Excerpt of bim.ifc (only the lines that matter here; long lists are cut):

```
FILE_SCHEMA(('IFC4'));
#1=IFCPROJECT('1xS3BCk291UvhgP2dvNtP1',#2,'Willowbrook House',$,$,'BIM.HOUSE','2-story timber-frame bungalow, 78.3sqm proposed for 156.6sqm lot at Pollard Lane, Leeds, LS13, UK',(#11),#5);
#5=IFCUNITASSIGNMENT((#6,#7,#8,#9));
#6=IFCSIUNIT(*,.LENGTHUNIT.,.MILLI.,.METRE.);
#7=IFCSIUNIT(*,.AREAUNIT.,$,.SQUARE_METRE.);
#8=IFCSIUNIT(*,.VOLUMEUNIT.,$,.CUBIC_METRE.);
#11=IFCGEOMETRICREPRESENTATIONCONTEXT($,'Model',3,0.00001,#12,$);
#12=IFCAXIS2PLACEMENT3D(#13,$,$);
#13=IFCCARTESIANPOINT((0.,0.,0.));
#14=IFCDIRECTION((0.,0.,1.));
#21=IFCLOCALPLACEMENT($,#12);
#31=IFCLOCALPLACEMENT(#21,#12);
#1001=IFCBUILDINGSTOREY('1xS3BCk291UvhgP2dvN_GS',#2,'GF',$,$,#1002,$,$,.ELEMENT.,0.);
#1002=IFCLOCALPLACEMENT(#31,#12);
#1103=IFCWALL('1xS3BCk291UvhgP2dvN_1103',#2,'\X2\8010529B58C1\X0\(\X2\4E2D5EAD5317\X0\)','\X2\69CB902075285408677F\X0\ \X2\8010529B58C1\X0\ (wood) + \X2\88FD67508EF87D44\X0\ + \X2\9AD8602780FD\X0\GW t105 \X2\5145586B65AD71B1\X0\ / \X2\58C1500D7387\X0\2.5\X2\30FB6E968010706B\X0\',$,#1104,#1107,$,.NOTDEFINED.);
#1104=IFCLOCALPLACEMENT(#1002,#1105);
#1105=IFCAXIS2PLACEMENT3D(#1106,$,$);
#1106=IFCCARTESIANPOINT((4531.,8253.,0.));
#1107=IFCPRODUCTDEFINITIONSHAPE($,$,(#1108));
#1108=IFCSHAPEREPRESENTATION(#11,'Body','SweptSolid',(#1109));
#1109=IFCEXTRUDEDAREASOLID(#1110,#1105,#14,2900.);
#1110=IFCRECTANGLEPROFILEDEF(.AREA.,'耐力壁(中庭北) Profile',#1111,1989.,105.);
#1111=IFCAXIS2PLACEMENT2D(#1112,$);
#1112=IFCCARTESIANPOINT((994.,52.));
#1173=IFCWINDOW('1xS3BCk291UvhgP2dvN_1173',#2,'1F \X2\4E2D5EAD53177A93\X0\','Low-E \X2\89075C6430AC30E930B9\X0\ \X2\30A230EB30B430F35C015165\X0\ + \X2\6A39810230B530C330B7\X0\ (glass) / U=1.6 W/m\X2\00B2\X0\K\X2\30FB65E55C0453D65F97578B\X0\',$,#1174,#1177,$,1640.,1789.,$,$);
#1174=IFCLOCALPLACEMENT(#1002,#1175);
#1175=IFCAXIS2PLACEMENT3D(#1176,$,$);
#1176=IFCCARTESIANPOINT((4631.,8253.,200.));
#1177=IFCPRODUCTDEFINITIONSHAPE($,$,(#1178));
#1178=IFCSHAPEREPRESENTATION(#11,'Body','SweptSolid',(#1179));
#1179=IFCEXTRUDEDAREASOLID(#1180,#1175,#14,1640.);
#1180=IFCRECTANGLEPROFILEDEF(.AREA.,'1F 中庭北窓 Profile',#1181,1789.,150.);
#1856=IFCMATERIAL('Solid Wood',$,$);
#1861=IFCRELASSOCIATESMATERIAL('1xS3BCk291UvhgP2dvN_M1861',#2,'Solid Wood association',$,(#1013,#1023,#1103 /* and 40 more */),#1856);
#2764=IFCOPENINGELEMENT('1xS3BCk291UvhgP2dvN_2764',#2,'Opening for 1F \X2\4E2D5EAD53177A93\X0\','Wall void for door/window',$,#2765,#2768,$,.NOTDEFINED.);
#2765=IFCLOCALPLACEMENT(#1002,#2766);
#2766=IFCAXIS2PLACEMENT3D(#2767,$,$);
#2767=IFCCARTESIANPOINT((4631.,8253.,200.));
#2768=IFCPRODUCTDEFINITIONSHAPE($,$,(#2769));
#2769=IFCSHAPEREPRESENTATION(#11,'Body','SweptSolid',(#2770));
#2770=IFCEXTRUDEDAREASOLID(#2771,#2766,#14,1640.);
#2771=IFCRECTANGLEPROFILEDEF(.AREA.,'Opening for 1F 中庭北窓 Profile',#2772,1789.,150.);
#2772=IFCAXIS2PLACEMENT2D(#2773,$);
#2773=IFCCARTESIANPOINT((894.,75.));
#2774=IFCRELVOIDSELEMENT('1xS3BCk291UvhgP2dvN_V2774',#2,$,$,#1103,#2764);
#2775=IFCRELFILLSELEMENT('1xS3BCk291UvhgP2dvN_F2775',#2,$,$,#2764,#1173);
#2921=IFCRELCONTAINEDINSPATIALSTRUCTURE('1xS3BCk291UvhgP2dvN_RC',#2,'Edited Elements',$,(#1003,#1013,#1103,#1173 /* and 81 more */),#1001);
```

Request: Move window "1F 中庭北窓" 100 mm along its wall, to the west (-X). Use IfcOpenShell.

```python
import ifcopenshell
import ifcopenshell.api.geometry
import ifcopenshell.util.placement
import ifcopenshell.util.unit

model = ifcopenshell.open("bim.ifc")
unit_scale = ifcopenshell.util.unit.calculate_unit_scale(model)

window = model.by_guid("1xS3BCk291UvhgP2dvN_1173")
opening = window.FillsVoids[0].RelatingOpeningElement
wall = opening.VoidsElements[0].RelatingBuildingElement

wall_matrix = ifcopenshell.util.placement.get_local_placement(wall.ObjectPlacement)
shift = wall_matrix[:3, 0] * -0.1 / unit_scale
before = ifcopenshell.util.placement.get_local_placement(window.ObjectPlacement)[:3, 3].copy()

# The window is not placed relative to its opening, so move both.
for product in (opening, window):
    matrix = ifcopenshell.util.placement.get_local_placement(product.ObjectPlacement)
    matrix[:3, 3] += shift
    ifcopenshell.api.geometry.edit_object_placement(model, product=product, matrix=matrix, is_si=False)

after = ifcopenshell.util.placement.get_local_placement(window.ObjectPlacement)[:3, 3]
print("window moved by", (after - before).round(3) + 0.0)

model.write("bim-out.ifc")
```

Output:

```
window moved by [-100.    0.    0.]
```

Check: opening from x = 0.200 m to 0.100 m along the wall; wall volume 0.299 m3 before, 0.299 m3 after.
